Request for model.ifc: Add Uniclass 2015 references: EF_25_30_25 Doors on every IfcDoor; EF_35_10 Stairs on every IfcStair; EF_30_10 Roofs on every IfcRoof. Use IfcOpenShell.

First a look at what the model holds.

```python
import ifcopenshell

model = ifcopenshell.open("model.ifc")
print(model.schema)
print("classifications:", [c.Name for c in model.by_type("IfcClassification")])
for ifc_class in ("IfcDoor", "IfcRoof", "IfcStair", "IfcWall", "IfcWindow"):
    print(ifc_class, len(model.by_type(ifc_class)))
```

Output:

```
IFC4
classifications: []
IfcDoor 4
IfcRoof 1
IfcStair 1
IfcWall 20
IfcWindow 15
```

```python
import ifcopenshell
import ifcopenshell.api.classification

model = ifcopenshell.open("model.ifc")

system = ifcopenshell.api.classification.add_classification(model, classification="Uniclass 2015")

codes = {
    "IfcDoor": ("EF_25_30_25", "Doors"),
    "IfcStair": ("EF_35_10", "Stairs"),
    "IfcRoof": ("EF_30_10", "Roofs"),
}
for ifc_class, (code, name) in codes.items():
    products = model.by_type(ifc_class)
    ifcopenshell.api.classification.add_reference(
        model, products=products, classification=system, identification=code, name=name
    )
    print(code, len(products))

model.write("model_edited.ifc")
```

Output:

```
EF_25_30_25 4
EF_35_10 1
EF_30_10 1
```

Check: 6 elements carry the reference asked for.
